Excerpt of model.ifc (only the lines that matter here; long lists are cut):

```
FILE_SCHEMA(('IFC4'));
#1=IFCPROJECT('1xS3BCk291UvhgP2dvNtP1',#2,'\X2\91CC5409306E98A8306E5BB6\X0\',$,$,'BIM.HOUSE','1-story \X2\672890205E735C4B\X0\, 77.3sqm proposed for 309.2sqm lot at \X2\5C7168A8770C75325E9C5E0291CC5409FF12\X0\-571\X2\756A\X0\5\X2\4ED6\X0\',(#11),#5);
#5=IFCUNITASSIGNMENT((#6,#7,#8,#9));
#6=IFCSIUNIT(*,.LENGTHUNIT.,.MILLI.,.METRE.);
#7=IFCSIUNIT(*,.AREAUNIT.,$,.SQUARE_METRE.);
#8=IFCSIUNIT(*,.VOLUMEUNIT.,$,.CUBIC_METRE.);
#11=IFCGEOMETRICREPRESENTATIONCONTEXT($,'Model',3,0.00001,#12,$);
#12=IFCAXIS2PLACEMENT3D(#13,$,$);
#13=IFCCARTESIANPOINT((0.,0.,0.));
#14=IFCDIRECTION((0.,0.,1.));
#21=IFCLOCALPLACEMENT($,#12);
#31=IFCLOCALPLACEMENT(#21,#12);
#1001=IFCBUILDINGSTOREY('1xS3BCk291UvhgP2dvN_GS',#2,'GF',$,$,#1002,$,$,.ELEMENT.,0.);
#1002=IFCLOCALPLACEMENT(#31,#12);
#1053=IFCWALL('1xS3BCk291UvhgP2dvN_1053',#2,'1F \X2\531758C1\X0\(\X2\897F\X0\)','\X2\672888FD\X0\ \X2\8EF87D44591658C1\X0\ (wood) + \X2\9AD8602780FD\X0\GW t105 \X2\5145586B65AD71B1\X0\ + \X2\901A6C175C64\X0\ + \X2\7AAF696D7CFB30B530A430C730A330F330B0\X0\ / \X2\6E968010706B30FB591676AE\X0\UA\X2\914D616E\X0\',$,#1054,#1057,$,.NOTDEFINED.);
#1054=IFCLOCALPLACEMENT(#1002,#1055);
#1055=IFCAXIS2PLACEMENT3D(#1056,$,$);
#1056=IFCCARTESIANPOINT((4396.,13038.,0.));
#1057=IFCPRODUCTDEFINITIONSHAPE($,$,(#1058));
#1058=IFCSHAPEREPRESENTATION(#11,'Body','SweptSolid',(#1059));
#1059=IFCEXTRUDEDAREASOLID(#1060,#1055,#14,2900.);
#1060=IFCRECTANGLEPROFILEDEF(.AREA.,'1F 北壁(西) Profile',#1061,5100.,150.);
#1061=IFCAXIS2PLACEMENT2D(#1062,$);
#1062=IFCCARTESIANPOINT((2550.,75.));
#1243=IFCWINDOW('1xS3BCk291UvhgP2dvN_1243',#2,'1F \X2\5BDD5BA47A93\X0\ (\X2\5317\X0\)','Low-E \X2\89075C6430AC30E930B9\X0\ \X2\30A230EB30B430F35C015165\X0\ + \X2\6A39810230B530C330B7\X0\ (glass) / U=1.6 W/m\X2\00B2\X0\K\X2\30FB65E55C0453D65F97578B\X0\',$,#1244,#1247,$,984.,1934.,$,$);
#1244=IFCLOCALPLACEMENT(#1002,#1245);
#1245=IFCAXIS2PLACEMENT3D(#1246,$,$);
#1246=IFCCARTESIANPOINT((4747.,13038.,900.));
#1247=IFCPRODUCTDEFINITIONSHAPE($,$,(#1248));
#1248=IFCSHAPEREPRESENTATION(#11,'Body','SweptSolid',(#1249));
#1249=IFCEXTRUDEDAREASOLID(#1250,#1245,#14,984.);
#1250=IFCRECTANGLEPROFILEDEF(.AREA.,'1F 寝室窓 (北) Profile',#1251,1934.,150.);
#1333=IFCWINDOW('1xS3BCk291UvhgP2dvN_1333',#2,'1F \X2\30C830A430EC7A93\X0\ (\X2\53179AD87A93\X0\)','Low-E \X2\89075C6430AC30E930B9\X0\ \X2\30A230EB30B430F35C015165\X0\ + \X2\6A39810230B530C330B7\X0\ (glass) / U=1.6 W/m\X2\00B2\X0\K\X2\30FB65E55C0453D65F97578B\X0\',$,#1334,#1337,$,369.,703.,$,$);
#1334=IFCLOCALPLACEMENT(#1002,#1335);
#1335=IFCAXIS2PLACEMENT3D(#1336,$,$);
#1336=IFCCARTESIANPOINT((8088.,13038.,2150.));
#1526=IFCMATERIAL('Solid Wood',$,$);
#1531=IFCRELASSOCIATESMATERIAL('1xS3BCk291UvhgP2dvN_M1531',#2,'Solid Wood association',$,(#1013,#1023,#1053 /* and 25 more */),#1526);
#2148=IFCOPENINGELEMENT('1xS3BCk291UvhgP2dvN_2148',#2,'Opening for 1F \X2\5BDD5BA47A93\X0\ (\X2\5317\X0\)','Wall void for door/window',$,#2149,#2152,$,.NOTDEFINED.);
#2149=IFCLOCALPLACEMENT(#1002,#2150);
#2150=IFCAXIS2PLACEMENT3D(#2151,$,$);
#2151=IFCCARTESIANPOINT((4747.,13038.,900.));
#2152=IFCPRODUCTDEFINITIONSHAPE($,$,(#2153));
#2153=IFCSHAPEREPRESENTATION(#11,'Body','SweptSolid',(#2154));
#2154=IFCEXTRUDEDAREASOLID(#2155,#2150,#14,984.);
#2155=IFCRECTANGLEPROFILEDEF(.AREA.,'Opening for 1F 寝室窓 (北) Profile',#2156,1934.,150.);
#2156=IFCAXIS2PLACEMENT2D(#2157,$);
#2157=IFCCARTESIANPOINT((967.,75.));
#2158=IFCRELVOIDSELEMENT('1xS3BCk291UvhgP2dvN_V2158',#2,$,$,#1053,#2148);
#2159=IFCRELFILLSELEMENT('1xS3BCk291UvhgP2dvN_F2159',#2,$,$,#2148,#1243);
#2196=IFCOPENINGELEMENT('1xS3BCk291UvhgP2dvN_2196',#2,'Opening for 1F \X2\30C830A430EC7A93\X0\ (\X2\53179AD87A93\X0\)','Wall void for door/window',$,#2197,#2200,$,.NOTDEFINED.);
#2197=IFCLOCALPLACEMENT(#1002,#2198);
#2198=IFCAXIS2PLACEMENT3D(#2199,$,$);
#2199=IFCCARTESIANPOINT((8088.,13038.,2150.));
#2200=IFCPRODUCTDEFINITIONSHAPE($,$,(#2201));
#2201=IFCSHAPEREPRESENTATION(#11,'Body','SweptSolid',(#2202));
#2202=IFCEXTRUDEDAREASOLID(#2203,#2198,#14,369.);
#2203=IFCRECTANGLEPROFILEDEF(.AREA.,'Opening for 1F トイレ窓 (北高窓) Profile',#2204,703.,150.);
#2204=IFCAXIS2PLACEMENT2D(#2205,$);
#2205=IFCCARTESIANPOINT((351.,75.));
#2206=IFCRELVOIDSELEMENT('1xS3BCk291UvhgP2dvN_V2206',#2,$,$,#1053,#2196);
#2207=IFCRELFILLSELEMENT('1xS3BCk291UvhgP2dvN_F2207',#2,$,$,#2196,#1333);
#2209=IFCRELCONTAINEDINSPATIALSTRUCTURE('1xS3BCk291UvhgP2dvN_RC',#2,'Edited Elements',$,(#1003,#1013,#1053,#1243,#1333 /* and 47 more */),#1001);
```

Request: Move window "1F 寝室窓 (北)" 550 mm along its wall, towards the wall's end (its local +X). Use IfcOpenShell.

```python
import ifcopenshell
import ifcopenshell.api.geometry
import ifcopenshell.util.placement
import ifcopenshell.util.unit

model = ifcopenshell.open("model.ifc")
unit_scale = ifcopenshell.util.unit.calculate_unit_scale(model)

window = model.by_id(1243)
opening = window.FillsVoids[0].RelatingOpeningElement
wall = opening.VoidsElements[0].RelatingBuildingElement

wall_matrix = ifcopenshell.util.placement.get_local_placement(wall.ObjectPlacement)
shift = wall_matrix[:3, 0] * 0.55 / unit_scale
before = ifcopenshell.util.placement.get_local_placement(window.ObjectPlacement)[:3, 3].copy()

# The window is not placed relative to its opening, so move both.
for product in (opening, window):
    matrix = ifcopenshell.util.placement.get_local_placement(product.ObjectPlacement)
    matrix[:3, 3] += shift
    ifcopenshell.api.geometry.edit_object_placement(model, product=product, matrix=matrix, is_si=False)

after = ifcopenshell.util.placement.get_local_placement(window.ObjectPlacement)[:3, 3]
print("window moved by", (after - before).round(3) + 0.0)

model.write("model_rev.ifc")
```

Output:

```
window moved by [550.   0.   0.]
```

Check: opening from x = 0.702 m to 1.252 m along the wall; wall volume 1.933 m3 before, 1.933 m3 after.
